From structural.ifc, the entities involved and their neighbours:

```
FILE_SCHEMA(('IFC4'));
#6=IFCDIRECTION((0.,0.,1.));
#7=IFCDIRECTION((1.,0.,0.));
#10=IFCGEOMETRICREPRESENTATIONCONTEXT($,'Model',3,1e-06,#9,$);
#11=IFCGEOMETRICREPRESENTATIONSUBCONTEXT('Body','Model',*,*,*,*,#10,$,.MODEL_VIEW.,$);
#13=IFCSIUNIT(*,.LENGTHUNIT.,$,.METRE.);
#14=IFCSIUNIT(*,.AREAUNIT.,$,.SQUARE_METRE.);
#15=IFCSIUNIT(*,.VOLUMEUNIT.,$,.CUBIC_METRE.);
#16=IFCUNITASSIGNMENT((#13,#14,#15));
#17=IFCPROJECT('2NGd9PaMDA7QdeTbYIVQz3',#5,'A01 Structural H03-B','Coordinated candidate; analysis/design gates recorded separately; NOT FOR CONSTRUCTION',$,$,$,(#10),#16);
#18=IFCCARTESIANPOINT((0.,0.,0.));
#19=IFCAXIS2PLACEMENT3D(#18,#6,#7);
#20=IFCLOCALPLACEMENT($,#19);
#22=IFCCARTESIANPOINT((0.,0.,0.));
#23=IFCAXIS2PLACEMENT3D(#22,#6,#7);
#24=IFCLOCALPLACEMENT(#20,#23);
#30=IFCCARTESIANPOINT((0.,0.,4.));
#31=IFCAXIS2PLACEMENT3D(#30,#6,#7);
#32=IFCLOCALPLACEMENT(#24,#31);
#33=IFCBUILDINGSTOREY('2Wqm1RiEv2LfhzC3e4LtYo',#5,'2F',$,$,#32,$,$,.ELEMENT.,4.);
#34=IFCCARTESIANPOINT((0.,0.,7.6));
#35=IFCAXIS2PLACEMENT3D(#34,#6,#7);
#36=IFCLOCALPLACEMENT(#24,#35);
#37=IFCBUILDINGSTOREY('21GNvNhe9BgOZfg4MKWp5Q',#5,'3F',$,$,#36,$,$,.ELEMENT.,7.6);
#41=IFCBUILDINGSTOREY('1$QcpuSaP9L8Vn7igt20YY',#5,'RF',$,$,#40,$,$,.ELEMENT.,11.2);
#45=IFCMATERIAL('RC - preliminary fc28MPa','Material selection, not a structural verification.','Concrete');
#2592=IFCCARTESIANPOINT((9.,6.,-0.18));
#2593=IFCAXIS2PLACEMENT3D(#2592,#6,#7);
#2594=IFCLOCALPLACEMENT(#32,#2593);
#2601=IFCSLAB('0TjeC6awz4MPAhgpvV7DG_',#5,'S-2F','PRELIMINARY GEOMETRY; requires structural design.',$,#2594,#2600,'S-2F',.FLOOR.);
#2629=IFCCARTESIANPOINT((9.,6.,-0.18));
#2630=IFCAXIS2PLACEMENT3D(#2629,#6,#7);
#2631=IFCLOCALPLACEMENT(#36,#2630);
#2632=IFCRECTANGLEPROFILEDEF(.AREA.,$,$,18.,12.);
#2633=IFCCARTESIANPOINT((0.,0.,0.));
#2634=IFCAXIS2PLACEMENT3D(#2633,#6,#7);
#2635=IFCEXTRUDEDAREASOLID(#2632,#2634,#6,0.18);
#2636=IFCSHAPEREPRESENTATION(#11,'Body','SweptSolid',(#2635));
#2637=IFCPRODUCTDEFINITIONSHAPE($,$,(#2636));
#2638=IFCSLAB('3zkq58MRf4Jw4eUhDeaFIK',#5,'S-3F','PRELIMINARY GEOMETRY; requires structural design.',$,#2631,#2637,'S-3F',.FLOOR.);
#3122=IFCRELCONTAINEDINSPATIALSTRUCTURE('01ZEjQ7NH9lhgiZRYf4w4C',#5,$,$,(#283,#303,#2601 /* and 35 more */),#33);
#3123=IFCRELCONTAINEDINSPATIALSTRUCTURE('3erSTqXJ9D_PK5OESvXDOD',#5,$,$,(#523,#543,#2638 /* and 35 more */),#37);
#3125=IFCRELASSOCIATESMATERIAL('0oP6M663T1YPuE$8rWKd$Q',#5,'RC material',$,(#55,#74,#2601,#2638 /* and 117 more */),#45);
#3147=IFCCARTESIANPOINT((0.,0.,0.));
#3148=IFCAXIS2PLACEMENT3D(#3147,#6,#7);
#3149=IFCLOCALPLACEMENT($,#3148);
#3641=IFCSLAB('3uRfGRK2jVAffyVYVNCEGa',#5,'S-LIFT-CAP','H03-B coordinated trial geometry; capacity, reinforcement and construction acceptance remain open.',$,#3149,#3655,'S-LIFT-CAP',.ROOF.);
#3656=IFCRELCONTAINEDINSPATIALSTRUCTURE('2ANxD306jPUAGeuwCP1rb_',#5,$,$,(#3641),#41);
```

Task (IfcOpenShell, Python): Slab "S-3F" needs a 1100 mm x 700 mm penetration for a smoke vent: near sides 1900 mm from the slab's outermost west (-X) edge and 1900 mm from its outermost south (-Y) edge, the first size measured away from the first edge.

```python
import numpy as np
import ifcopenshell
import ifcopenshell.api.feature
import ifcopenshell.api.geometry
import ifcopenshell.api.root
import ifcopenshell.geom
import ifcopenshell.util.placement
import ifcopenshell.util.representation
import ifcopenshell.util.shape
import ifcopenshell.util.unit

model = ifcopenshell.open("structural.ifc")
unit_scale = ifcopenshell.util.unit.calculate_unit_scale(model)
settings = ifcopenshell.geom.settings()


def volume(element):
    """Net volume in cubic metres, openings subtracted."""
    shape = ifcopenshell.geom.create_shape(settings, element)
    return ifcopenshell.util.shape.get_volume(shape.geometry)


slab = model.by_guid("3zkq58MRf4Jw4eUhDeaFIK")
before = volume(slab)

# Extent in the slab's own axes, in metres. The edges named are its -X and -Y sides.
slab_shape = ifcopenshell.geom.create_shape(settings, slab)
vertices = ifcopenshell.util.shape.get_vertices(slab_shape.geometry)
x_min, y_min, bottom = vertices.min(axis=0)
top = vertices[:, 2].max()

opening = ifcopenshell.api.root.create_entity(model, ifc_class="IfcOpeningElement", name="Smoke vent opening", predefined_type="OPENING")
context = ifcopenshell.util.representation.get_context(model, "Model", "Body", "MODEL_VIEW")
width, depth = 1.1, 0.7
outline = [(0.0, 0.0), (width, 0.0), (width, depth), (0.0, depth), (0.0, 0.0)]
# Overshoot both faces by 50 mm so the cut is clean.
shape = ifcopenshell.api.geometry.add_slab_representation(
    model, context=context, depth=top - bottom + 0.1, polyline=outline
)
ifcopenshell.api.geometry.assign_representation(model, product=opening, representation=shape)

matrix = ifcopenshell.util.placement.get_local_placement(slab.ObjectPlacement)
matrix[:, 3] = matrix @ np.append(np.array([x_min + 1.9, y_min + 1.9, bottom - 0.05]) / unit_scale, 1.0)
ifcopenshell.api.geometry.edit_object_placement(model, product=opening, matrix=matrix, is_si=False)
ifcopenshell.api.feature.add_feature(model, feature=opening, element=slab)

after = volume(slab)

print(f"slab volume {before:.3f} -> {after:.3f} m3")

model.write("structural_updated.ifc")
```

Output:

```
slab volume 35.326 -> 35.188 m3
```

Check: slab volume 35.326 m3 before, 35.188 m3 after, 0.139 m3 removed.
